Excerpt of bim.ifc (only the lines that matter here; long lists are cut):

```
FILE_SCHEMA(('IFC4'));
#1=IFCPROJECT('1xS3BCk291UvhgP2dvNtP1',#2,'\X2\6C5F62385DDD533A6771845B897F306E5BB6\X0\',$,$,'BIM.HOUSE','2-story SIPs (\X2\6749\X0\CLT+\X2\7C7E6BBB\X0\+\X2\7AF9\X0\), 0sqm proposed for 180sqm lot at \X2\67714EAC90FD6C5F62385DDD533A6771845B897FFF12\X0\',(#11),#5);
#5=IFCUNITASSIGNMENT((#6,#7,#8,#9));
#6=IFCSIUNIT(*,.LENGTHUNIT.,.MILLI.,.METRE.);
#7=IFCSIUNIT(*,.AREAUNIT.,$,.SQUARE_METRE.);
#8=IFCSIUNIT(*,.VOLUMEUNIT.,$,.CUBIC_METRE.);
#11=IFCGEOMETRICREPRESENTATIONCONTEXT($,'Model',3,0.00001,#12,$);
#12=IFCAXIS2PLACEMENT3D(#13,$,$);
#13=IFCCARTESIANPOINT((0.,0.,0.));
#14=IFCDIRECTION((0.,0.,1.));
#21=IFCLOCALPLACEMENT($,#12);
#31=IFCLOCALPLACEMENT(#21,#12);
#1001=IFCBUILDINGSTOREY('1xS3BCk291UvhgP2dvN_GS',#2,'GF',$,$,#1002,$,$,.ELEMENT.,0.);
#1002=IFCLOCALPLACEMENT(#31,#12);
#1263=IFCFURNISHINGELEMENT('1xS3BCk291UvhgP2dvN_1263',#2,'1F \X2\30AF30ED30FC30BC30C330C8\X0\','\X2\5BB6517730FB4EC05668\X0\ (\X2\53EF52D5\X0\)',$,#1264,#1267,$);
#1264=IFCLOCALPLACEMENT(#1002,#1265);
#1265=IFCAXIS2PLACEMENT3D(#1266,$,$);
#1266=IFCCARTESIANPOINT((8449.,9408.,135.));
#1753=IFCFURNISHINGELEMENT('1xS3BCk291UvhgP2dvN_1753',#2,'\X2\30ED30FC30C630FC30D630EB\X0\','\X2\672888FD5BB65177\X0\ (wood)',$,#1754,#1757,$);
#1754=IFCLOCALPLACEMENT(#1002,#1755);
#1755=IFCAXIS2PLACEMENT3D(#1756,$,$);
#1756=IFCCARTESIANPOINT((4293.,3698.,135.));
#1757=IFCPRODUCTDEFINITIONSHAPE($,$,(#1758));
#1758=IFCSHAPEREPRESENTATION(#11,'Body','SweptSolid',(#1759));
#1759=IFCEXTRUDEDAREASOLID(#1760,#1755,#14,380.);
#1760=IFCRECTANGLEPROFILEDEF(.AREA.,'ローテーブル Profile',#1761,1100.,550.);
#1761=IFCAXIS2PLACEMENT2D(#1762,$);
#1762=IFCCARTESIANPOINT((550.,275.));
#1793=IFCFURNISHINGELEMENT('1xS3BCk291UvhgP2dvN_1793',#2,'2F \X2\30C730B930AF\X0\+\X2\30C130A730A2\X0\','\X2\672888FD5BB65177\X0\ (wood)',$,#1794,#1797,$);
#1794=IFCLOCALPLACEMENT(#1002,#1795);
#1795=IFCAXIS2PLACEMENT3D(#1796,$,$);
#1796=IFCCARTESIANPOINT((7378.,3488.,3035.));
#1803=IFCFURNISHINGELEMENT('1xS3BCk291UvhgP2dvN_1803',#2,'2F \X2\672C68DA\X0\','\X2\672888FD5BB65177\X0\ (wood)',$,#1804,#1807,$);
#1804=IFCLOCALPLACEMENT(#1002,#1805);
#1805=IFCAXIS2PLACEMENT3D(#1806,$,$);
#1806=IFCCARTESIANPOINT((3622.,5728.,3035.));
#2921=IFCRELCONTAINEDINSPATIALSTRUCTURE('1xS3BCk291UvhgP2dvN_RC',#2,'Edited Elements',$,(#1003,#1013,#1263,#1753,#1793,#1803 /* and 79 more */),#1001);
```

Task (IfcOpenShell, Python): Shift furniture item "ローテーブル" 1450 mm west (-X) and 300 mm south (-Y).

```python
import ifcopenshell
import ifcopenshell.api.geometry
import ifcopenshell.util.placement
import ifcopenshell.util.unit

model = ifcopenshell.open("bim.ifc")
unit_scale = ifcopenshell.util.unit.calculate_unit_scale(model)

item = model.by_guid("1xS3BCk291UvhgP2dvN_1753")
matrix = ifcopenshell.util.placement.get_local_placement(item.ObjectPlacement)
matrix[0, 3] -= 1.45 / unit_scale
matrix[1, 3] -= 0.3 / unit_scale
ifcopenshell.api.geometry.edit_object_placement(model, product=item, matrix=matrix, is_si=False)

print(ifcopenshell.util.placement.get_local_placement(item.ObjectPlacement).round(3) + 0.0)

model.write("bim_v2.ifc")
```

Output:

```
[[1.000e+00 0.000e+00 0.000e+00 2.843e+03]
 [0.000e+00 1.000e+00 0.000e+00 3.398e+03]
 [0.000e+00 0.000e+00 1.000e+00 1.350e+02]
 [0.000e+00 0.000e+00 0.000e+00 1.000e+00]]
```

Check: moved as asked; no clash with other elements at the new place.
